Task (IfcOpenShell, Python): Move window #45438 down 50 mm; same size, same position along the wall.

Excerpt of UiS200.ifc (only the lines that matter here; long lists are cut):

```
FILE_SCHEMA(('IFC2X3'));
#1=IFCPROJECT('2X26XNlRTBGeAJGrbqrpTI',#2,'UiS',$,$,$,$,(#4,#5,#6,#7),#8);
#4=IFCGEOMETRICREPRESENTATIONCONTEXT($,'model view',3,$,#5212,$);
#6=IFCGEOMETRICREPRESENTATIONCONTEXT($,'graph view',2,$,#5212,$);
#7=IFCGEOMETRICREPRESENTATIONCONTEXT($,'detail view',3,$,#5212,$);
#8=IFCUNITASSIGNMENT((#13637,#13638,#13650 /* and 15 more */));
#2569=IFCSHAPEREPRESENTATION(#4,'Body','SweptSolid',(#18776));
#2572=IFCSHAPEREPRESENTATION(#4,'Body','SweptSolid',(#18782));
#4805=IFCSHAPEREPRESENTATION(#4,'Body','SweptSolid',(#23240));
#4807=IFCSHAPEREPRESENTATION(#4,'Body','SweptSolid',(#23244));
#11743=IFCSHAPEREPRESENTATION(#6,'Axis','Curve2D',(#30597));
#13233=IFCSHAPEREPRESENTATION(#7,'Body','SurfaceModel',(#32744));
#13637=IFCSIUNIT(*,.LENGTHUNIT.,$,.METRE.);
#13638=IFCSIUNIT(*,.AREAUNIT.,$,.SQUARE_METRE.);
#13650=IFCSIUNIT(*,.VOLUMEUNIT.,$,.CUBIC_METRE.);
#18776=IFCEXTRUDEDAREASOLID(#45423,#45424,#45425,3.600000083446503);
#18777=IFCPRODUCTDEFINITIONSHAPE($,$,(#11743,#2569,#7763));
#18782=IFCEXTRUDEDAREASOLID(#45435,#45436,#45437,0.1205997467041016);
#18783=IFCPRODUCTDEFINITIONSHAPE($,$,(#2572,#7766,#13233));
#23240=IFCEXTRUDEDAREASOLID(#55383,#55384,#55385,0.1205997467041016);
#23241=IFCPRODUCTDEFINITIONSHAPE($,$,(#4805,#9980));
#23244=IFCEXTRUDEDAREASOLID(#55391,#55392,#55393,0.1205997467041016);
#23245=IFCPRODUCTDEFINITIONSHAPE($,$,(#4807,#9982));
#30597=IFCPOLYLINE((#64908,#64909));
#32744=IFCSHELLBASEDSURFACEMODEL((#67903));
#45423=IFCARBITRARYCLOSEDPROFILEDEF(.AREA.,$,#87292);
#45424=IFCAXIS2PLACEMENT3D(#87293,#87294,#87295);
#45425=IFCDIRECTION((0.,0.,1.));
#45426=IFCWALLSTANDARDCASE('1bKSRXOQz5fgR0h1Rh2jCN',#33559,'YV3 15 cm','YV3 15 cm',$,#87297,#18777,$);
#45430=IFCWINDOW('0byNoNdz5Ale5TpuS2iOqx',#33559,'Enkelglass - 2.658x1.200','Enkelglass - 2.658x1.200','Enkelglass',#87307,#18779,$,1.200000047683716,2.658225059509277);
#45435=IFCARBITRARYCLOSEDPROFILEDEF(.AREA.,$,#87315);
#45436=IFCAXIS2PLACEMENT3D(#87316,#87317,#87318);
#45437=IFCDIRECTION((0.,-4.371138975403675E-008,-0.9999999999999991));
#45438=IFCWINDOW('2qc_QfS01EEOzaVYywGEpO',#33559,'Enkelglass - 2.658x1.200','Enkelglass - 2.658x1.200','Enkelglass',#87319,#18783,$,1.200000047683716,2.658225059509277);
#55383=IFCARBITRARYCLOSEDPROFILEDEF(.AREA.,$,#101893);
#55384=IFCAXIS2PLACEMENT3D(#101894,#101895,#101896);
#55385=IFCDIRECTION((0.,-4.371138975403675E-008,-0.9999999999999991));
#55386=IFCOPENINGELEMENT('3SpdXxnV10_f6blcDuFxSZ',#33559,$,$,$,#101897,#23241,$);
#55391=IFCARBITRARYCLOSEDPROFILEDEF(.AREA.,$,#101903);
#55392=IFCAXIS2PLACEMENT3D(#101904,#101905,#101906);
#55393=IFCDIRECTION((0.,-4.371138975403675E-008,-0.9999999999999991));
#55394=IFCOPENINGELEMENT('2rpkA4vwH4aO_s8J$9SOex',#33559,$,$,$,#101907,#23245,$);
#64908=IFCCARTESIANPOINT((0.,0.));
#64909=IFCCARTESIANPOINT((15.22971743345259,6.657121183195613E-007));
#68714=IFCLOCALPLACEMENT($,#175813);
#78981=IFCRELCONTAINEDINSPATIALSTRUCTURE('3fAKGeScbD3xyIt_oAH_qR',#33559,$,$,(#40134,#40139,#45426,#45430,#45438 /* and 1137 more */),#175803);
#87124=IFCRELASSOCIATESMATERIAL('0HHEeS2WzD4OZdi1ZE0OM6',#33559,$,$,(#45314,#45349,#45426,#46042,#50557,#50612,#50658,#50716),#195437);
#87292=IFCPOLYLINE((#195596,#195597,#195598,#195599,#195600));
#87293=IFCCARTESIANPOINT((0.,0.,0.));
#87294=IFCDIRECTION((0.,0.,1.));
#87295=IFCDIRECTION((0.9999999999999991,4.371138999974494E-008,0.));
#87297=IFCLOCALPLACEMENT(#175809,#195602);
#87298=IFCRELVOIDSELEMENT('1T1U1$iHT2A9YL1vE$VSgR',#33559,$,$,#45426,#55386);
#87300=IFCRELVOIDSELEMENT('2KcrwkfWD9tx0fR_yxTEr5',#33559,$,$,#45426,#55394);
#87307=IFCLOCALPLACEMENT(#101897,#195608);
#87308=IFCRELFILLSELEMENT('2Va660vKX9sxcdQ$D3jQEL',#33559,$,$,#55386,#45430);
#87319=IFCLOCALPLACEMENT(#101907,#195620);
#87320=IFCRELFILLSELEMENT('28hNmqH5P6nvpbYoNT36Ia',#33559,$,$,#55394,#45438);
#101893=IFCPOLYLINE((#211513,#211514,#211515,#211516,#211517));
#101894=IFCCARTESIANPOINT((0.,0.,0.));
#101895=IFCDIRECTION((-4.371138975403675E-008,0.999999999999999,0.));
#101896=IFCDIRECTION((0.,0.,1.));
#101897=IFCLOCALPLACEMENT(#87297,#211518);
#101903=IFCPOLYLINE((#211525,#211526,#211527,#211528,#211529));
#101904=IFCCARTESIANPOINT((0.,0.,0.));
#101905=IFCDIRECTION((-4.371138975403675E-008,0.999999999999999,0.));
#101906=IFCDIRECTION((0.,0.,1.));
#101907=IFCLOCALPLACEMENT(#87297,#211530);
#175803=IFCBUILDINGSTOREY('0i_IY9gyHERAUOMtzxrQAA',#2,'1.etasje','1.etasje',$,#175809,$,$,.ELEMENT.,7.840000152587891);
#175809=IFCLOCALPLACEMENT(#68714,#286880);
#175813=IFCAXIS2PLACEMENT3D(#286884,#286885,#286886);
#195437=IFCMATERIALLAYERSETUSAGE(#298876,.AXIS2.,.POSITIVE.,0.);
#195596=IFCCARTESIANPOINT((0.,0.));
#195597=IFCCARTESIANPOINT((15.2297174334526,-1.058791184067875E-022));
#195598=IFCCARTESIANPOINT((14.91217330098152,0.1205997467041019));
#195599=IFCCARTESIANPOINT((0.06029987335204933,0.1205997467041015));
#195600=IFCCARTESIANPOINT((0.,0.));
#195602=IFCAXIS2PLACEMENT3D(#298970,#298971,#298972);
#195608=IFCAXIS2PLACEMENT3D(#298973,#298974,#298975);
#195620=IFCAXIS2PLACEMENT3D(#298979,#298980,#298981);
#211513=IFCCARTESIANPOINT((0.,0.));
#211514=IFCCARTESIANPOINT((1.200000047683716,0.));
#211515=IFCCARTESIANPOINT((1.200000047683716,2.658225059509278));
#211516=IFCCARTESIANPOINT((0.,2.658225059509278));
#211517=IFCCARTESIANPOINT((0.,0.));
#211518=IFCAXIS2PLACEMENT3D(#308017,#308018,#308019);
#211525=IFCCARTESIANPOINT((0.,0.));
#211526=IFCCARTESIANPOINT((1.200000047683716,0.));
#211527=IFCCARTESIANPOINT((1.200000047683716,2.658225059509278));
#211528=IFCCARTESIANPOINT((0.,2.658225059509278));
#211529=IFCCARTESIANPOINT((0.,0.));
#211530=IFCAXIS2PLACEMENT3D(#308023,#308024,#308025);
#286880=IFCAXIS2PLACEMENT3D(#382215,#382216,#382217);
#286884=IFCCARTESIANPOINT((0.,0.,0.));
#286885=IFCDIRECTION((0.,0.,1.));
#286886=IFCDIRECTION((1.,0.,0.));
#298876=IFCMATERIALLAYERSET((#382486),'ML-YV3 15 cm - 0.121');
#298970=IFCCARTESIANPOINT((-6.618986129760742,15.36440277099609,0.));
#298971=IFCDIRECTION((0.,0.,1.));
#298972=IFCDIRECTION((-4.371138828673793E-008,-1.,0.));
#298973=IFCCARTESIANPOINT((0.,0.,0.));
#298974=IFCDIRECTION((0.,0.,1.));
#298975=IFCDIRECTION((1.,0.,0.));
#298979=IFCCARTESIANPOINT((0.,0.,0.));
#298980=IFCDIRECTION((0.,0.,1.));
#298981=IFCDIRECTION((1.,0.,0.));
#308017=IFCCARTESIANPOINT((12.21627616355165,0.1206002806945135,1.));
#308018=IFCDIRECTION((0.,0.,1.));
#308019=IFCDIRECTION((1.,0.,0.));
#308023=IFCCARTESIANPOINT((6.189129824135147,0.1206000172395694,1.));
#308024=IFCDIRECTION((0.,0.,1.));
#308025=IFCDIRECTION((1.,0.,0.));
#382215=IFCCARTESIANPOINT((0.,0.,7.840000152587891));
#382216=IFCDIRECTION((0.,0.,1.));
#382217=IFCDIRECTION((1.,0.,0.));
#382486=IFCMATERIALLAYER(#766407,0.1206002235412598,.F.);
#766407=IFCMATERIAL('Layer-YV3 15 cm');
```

```python
import numpy as np
import ifcopenshell
import ifcopenshell.api.geometry
import ifcopenshell.util.placement
import ifcopenshell.util.unit

model = ifcopenshell.open("UiS200.ifc")
unit_scale = ifcopenshell.util.unit.calculate_unit_scale(model)

window = model.by_guid("2qc_QfS01EEOzaVYywGEpO")
opening = window.FillsVoids[0].RelatingOpeningElement
dz = -0.05 / unit_scale

shift = np.array([0.0, 0.0, dz])
# The window is placed relative to its opening, so it follows when the opening moves.
matrix = ifcopenshell.util.placement.get_local_placement(opening.ObjectPlacement)
matrix[:3, 3] += shift
ifcopenshell.api.geometry.edit_object_placement(
    model, product=opening, matrix=matrix, is_si=False, should_transform_children=True
)

print(f"moved by {dz * unit_scale:+.3f} m")

model.write("UiS200_updated.ifc")
```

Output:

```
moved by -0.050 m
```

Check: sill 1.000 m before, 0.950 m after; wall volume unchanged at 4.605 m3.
